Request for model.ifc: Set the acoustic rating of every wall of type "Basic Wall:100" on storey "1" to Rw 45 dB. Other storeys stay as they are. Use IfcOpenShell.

First a look at what the model holds.

```python
import ifcopenshell
import ifcopenshell.util.element

model = ifcopenshell.open("model.ifc")
print(model.schema)
storey = next(s for s in model.by_type("IfcBuildingStorey") if s.Name == "1")
walls = [e for e in ifcopenshell.util.element.get_decomposition(storey) if e.is_a("IfcWall")]
seen = {}
for e in walls:
    element_type = ifcopenshell.util.element.get_type(e)
    key = (element_type.Name if element_type != e and element_type else None, ifcopenshell.util.element.get_pset(e, "Pset_WallCommon", "AcousticRating"))
    seen[key] = seen.get(key, 0) + 1
for (name, value), count in sorted(seen.items(), key=str):
    print(count, "x", name, "|", value)
```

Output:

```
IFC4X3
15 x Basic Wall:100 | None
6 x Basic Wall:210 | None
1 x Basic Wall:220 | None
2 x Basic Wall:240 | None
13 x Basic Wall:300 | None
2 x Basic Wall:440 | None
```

```python
import ifcopenshell
import ifcopenshell.api.pset
import ifcopenshell.util.element

model = ifcopenshell.open("model.ifc")

storey = next(s for s in model.by_type("IfcBuildingStorey") if s.Name == "1")
walls = [e for e in ifcopenshell.util.element.get_decomposition(storey) if e.is_a("IfcWall")]

count = 0
for e in walls:
    element_type = ifcopenshell.util.element.get_type(e)
    if element_type in (None, e) or element_type.Name != "Basic Wall:100":
        continue
    # add_pset returns the element's existing set when there is one.
    pset = ifcopenshell.api.pset.add_pset(model, product=e, name="Pset_WallCommon")
    ifcopenshell.api.pset.edit_pset(model, pset=pset, properties={"AcousticRating": "Rw 45 dB"})
    count += 1

print(count, "walls updated")

model.write("model_updated.ifc")
```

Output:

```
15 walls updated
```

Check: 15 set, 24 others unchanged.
